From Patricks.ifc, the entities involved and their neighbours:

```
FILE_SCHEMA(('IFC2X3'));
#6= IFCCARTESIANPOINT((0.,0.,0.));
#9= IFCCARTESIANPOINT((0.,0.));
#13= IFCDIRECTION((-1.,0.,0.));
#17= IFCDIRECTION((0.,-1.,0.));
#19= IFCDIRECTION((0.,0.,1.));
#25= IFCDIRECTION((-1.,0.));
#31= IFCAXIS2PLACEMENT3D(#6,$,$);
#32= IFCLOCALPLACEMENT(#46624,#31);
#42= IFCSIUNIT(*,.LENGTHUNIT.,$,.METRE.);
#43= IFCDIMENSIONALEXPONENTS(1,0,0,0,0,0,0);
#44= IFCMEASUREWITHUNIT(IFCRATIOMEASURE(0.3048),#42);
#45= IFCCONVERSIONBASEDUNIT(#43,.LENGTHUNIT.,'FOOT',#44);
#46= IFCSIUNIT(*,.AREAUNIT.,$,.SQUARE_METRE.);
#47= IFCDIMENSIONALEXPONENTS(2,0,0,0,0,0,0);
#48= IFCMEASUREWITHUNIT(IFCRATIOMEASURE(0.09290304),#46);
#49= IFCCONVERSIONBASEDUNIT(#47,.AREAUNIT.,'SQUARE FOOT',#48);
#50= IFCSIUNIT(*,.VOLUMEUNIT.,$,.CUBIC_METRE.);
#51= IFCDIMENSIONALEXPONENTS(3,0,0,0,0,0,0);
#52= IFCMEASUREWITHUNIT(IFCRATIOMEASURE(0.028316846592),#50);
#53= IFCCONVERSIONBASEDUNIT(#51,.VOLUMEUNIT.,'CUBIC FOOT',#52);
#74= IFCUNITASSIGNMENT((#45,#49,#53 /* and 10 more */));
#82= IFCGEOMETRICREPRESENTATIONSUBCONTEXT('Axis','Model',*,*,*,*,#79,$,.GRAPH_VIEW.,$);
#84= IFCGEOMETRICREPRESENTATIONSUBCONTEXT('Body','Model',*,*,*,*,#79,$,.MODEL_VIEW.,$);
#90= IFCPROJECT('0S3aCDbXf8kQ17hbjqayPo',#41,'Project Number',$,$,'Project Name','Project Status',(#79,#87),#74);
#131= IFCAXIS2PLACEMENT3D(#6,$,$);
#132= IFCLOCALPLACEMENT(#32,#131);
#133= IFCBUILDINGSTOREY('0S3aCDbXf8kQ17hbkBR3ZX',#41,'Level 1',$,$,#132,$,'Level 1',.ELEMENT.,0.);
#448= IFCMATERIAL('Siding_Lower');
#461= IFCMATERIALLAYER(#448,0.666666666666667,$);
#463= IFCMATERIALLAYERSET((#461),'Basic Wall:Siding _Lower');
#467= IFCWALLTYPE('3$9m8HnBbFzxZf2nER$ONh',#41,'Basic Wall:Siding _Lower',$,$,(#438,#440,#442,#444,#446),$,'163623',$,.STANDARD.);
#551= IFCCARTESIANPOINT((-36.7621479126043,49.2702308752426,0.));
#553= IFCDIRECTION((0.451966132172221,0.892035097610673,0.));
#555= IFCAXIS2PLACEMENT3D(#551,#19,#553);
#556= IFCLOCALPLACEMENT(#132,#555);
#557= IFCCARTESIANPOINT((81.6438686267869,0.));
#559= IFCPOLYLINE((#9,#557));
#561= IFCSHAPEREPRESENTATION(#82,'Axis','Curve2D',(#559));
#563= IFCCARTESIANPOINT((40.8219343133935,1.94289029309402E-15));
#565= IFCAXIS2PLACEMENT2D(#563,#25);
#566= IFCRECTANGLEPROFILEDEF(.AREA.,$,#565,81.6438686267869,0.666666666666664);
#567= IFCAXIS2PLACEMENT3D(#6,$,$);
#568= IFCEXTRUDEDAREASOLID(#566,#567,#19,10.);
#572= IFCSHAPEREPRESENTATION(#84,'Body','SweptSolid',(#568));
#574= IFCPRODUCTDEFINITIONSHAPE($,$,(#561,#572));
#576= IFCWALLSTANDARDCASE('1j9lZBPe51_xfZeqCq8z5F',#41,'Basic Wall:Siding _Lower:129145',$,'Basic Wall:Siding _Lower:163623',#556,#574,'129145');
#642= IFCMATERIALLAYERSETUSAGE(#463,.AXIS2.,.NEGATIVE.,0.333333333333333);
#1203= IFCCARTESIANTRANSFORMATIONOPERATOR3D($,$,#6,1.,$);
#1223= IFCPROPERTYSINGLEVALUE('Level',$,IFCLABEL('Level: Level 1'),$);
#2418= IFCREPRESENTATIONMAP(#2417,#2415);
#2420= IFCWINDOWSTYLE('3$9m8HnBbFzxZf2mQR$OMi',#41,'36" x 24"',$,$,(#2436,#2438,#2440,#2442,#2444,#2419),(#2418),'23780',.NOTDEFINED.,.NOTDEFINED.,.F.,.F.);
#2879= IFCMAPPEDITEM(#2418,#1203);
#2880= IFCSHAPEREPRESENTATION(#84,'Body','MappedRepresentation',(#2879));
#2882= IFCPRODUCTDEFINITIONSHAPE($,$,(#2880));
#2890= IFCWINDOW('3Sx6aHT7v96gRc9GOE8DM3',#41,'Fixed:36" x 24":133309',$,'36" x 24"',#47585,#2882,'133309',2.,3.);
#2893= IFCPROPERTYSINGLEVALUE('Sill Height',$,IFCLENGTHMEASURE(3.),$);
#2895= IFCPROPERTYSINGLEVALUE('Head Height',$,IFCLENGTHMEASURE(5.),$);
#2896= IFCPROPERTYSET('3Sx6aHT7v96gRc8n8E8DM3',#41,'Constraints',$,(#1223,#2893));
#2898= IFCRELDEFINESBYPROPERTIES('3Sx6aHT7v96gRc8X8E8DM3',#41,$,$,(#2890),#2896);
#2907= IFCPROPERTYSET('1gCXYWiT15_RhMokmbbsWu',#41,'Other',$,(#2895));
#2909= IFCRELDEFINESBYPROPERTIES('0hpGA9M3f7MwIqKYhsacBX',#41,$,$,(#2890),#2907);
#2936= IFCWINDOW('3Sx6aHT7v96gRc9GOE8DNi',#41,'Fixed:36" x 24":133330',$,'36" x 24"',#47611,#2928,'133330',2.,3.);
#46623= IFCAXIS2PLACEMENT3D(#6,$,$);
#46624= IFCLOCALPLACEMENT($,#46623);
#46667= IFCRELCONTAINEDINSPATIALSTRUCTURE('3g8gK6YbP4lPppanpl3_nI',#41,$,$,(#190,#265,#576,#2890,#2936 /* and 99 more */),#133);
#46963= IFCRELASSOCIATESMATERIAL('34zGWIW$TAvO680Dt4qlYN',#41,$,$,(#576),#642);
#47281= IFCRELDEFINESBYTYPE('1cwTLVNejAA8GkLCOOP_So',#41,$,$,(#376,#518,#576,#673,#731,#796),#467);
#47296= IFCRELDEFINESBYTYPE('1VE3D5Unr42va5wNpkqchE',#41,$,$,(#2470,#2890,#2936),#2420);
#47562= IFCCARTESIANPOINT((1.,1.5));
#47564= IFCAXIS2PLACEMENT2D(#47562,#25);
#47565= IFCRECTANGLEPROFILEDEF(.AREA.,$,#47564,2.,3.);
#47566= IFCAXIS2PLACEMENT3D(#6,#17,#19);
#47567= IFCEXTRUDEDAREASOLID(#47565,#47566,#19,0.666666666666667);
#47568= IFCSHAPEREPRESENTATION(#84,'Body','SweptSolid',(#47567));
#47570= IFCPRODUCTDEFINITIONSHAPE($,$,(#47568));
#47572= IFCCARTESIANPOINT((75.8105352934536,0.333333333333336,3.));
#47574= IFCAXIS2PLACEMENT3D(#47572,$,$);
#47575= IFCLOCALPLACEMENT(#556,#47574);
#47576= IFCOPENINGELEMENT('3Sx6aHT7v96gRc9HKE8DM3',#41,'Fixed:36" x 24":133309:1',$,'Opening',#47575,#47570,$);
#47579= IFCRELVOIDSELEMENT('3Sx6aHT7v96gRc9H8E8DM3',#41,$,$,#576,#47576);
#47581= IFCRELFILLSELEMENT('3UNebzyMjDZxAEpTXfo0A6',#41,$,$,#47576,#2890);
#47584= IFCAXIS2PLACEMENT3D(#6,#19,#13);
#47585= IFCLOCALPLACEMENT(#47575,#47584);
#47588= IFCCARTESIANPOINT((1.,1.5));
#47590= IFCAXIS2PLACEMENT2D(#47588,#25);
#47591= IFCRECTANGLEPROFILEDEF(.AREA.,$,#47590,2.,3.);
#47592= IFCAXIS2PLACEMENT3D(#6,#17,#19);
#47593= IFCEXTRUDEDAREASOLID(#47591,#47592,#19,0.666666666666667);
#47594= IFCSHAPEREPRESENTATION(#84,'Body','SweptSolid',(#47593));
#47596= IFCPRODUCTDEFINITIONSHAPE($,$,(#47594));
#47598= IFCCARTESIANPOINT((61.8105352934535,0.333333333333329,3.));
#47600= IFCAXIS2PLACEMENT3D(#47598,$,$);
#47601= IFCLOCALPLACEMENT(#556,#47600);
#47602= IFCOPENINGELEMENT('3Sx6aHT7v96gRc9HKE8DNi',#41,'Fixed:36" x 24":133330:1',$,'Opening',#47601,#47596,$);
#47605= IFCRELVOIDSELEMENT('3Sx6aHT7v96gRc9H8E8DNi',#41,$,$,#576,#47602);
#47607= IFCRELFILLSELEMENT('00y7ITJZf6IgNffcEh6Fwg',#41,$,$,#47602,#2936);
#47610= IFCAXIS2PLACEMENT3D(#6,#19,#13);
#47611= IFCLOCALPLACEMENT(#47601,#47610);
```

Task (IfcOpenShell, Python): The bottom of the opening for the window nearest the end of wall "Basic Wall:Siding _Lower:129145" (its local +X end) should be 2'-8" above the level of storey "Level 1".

```python
import numpy as np
import ifcopenshell
import ifcopenshell.api.geometry
import ifcopenshell.api.pset
import ifcopenshell.geom
import ifcopenshell.util.element
import ifcopenshell.util.placement
import ifcopenshell.util.shape
import ifcopenshell.util.unit

model = ifcopenshell.open("Patricks.ifc")
unit_scale = ifcopenshell.util.unit.calculate_unit_scale(model)

window = model.by_guid("3Sx6aHT7v96gRc9GOE8DM3")
opening = window.FillsVoids[0].RelatingOpeningElement
storey = ifcopenshell.util.element.get_container(window, ifc_class="IfcBuildingStorey")
level = ifcopenshell.util.placement.get_local_placement(storey.ObjectPlacement)[2, 3]

# The opening's origin need not be at the sill, so measure its lowest point.
shape = ifcopenshell.geom.create_shape(ifcopenshell.geom.settings(), opening)
bottom = ifcopenshell.util.shape.get_shape_bottom_elevation(shape, shape.geometry) / unit_scale
dz = level + 32 * 0.0254 / unit_scale - bottom

shift = np.array([0.0, 0.0, dz])
# The window is placed relative to its opening, so it follows when the opening moves.
matrix = ifcopenshell.util.placement.get_local_placement(opening.ObjectPlacement)
matrix[:3, 3] += shift
ifcopenshell.api.geometry.edit_object_placement(
    model, product=opening, matrix=matrix, is_si=False, should_transform_children=True
)

# Keep the stored heights in step.
pset = model.by_id(ifcopenshell.util.element.get_pset(window, "Constraints", should_inherit=False)["id"])
ifcopenshell.api.pset.edit_pset(model, pset=pset, properties={
    "Sill Height": model.create_entity("IfcLengthMeasure", ifcopenshell.util.element.get_pset(window, "Constraints", "Sill Height") + dz),
})
pset = model.by_id(ifcopenshell.util.element.get_pset(window, "Other", should_inherit=False)["id"])
ifcopenshell.api.pset.edit_pset(model, pset=pset, properties={
    "Head Height": model.create_entity("IfcLengthMeasure", ifcopenshell.util.element.get_pset(window, "Other", "Head Height") + dz),
})

print(f"moved by {dz * unit_scale:+.3f} m")

model.write("Patricks_updated.ifc")
```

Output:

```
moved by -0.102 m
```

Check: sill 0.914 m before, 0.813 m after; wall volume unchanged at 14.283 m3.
